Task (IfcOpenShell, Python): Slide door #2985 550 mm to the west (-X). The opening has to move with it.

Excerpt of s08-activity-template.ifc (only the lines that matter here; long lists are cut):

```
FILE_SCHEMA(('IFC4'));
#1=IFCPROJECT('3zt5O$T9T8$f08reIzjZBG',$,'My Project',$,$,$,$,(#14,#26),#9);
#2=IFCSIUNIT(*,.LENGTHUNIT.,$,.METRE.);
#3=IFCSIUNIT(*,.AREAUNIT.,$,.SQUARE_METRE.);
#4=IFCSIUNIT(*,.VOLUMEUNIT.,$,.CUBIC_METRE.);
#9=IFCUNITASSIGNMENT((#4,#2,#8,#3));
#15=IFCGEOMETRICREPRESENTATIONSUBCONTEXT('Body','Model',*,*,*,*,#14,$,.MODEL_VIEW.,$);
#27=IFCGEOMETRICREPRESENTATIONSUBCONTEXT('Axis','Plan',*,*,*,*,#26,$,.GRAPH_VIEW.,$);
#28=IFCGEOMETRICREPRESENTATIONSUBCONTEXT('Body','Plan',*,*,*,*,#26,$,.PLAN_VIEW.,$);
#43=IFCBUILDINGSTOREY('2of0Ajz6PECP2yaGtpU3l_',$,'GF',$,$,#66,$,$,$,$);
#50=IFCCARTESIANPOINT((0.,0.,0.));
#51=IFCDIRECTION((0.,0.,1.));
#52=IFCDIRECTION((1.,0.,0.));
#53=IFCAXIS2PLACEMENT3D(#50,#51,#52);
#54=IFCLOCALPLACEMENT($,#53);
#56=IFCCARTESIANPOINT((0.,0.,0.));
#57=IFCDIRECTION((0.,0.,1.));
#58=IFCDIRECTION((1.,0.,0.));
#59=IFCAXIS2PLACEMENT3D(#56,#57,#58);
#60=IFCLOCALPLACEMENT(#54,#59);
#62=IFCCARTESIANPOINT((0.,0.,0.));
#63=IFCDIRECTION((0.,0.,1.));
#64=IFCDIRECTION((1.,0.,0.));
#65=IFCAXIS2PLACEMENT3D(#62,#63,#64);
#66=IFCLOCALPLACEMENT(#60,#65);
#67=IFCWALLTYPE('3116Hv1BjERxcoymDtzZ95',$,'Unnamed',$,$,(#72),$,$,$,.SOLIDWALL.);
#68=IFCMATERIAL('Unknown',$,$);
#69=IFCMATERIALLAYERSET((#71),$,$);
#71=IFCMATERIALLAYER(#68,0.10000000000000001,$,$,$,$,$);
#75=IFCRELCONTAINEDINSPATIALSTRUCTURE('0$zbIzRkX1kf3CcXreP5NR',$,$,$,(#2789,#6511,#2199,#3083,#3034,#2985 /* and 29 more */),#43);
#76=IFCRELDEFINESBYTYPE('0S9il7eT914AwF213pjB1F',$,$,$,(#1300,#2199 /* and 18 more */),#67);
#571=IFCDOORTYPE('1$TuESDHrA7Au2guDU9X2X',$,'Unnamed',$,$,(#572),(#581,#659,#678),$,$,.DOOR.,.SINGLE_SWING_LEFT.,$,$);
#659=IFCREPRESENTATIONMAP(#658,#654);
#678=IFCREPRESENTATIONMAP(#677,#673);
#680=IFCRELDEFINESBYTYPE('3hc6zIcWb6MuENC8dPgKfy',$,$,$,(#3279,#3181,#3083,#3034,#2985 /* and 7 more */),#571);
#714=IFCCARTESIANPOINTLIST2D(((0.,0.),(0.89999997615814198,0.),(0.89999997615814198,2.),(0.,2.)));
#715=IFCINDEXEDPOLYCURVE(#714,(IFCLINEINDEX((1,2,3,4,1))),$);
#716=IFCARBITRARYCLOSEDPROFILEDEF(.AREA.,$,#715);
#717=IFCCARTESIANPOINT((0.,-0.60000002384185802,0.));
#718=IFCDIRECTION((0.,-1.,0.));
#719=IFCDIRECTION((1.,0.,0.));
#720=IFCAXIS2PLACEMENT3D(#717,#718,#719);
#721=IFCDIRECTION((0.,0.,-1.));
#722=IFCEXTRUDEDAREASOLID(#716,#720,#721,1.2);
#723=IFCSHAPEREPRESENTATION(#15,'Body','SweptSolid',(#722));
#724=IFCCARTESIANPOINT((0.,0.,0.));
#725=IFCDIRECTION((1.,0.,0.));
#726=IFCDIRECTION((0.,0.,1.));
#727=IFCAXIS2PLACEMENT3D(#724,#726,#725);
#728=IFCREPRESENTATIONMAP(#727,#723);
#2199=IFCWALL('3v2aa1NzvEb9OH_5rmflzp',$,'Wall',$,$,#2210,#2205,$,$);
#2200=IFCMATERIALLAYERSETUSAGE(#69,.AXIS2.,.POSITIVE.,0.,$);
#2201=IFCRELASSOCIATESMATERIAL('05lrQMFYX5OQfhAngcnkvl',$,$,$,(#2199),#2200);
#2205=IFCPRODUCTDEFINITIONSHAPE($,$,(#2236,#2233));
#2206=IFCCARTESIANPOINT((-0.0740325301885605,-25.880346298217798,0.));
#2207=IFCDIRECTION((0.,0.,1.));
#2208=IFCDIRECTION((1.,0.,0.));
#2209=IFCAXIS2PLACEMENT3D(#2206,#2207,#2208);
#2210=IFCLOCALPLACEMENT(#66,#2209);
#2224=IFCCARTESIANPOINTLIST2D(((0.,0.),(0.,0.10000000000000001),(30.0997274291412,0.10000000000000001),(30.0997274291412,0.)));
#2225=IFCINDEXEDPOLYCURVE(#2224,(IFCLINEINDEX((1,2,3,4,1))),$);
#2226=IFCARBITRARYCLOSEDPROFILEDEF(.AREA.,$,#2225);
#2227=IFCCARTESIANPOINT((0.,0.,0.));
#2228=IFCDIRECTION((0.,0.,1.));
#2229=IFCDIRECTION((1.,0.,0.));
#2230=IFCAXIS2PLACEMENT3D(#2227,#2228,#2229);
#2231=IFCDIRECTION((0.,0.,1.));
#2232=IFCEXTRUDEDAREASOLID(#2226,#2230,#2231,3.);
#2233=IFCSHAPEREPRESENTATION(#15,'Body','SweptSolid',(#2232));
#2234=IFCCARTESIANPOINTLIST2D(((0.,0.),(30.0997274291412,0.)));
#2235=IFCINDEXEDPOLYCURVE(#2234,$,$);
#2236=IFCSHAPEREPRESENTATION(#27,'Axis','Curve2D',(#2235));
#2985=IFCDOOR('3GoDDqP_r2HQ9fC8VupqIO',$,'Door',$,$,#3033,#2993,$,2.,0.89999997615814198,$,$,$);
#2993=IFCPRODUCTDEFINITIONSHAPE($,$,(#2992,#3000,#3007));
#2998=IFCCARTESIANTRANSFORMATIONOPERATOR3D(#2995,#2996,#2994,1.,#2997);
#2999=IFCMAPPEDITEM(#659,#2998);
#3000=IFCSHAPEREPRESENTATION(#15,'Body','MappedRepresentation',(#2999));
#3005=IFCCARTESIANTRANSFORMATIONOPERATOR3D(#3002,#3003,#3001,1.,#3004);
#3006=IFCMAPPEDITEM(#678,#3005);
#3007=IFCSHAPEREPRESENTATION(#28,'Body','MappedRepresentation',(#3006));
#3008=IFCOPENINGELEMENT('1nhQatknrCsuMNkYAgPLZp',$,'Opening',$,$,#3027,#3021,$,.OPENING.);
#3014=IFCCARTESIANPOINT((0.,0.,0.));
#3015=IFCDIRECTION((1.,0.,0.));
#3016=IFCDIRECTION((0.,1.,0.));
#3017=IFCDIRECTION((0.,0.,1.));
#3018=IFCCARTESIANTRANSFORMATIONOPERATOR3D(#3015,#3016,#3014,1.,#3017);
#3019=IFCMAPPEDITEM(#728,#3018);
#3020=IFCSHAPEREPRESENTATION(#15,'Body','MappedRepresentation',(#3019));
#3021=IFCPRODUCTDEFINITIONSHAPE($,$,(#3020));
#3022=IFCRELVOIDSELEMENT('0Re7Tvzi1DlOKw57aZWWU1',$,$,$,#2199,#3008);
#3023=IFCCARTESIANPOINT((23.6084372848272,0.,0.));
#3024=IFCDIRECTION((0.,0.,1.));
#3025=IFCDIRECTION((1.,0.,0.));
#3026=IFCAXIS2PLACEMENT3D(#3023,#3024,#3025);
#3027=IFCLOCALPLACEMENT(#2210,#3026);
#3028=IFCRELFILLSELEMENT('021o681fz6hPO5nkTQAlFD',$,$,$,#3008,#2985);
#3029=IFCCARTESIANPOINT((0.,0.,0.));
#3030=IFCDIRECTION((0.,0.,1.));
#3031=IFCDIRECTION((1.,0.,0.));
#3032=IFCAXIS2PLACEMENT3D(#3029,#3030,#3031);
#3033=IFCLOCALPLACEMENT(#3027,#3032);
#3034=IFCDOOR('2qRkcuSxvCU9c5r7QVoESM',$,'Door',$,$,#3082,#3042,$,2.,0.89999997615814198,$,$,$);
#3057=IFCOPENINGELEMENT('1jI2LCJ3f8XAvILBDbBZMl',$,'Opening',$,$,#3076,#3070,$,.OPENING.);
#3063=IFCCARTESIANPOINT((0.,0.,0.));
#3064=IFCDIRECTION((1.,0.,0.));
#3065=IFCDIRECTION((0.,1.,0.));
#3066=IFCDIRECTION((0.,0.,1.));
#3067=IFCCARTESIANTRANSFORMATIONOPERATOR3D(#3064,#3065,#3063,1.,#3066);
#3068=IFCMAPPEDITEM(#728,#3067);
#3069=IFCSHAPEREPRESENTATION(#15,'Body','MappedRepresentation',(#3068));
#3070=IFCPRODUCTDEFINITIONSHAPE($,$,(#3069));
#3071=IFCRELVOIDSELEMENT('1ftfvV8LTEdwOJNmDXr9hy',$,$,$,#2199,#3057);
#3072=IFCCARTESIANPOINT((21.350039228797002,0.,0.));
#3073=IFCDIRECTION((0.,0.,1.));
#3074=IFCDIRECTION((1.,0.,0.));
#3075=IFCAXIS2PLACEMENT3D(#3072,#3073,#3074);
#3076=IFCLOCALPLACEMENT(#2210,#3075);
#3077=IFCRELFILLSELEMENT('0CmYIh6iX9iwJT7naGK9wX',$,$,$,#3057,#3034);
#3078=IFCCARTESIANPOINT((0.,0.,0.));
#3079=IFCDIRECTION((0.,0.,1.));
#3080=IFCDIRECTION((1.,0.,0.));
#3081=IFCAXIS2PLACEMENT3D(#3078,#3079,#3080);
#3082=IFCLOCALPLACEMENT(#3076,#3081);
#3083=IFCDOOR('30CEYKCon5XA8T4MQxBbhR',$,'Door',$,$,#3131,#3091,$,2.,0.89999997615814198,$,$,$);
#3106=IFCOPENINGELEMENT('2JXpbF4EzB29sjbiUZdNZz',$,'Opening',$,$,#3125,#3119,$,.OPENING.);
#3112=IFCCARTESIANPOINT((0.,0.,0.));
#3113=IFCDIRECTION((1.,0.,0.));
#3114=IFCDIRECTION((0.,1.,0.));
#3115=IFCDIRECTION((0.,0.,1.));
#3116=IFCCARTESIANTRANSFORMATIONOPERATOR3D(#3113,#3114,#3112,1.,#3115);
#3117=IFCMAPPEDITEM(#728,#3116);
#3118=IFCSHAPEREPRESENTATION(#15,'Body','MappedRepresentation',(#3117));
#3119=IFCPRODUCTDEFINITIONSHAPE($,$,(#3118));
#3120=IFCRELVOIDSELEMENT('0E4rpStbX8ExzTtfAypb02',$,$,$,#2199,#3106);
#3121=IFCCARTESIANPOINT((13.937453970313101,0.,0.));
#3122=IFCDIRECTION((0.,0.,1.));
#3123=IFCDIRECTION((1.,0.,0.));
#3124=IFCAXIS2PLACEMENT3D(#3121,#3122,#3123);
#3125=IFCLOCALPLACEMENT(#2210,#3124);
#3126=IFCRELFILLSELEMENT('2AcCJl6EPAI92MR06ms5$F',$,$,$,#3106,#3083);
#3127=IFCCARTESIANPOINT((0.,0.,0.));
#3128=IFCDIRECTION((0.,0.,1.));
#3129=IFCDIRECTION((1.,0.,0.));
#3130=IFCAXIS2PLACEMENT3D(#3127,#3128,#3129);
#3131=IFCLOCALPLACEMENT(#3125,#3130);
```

```python
import ifcopenshell
import ifcopenshell.api.geometry
import ifcopenshell.util.placement
import ifcopenshell.util.unit

model = ifcopenshell.open("s08-activity-template.ifc")
unit_scale = ifcopenshell.util.unit.calculate_unit_scale(model)

door = model.by_id(2985)
opening = door.FillsVoids[0].RelatingOpeningElement
wall = opening.VoidsElements[0].RelatingBuildingElement

wall_matrix = ifcopenshell.util.placement.get_local_placement(wall.ObjectPlacement)
shift = wall_matrix[:3, 0] * -0.55 / unit_scale
before = ifcopenshell.util.placement.get_local_placement(door.ObjectPlacement)[:3, 3].copy()

# The door is placed relative to its opening, so it follows when the opening moves.
matrix = ifcopenshell.util.placement.get_local_placement(opening.ObjectPlacement)
matrix[:3, 3] += shift
ifcopenshell.api.geometry.edit_object_placement(
    model, product=opening, matrix=matrix, is_si=False, should_transform_children=True
)

after = ifcopenshell.util.placement.get_local_placement(door.ObjectPlacement)[:3, 3]
print("door moved by", (after - before).round(3) + 0.0)

model.write("s08-activity-template_edited.ifc")
```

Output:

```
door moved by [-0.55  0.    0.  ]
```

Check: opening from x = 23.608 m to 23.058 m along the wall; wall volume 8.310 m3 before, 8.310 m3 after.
